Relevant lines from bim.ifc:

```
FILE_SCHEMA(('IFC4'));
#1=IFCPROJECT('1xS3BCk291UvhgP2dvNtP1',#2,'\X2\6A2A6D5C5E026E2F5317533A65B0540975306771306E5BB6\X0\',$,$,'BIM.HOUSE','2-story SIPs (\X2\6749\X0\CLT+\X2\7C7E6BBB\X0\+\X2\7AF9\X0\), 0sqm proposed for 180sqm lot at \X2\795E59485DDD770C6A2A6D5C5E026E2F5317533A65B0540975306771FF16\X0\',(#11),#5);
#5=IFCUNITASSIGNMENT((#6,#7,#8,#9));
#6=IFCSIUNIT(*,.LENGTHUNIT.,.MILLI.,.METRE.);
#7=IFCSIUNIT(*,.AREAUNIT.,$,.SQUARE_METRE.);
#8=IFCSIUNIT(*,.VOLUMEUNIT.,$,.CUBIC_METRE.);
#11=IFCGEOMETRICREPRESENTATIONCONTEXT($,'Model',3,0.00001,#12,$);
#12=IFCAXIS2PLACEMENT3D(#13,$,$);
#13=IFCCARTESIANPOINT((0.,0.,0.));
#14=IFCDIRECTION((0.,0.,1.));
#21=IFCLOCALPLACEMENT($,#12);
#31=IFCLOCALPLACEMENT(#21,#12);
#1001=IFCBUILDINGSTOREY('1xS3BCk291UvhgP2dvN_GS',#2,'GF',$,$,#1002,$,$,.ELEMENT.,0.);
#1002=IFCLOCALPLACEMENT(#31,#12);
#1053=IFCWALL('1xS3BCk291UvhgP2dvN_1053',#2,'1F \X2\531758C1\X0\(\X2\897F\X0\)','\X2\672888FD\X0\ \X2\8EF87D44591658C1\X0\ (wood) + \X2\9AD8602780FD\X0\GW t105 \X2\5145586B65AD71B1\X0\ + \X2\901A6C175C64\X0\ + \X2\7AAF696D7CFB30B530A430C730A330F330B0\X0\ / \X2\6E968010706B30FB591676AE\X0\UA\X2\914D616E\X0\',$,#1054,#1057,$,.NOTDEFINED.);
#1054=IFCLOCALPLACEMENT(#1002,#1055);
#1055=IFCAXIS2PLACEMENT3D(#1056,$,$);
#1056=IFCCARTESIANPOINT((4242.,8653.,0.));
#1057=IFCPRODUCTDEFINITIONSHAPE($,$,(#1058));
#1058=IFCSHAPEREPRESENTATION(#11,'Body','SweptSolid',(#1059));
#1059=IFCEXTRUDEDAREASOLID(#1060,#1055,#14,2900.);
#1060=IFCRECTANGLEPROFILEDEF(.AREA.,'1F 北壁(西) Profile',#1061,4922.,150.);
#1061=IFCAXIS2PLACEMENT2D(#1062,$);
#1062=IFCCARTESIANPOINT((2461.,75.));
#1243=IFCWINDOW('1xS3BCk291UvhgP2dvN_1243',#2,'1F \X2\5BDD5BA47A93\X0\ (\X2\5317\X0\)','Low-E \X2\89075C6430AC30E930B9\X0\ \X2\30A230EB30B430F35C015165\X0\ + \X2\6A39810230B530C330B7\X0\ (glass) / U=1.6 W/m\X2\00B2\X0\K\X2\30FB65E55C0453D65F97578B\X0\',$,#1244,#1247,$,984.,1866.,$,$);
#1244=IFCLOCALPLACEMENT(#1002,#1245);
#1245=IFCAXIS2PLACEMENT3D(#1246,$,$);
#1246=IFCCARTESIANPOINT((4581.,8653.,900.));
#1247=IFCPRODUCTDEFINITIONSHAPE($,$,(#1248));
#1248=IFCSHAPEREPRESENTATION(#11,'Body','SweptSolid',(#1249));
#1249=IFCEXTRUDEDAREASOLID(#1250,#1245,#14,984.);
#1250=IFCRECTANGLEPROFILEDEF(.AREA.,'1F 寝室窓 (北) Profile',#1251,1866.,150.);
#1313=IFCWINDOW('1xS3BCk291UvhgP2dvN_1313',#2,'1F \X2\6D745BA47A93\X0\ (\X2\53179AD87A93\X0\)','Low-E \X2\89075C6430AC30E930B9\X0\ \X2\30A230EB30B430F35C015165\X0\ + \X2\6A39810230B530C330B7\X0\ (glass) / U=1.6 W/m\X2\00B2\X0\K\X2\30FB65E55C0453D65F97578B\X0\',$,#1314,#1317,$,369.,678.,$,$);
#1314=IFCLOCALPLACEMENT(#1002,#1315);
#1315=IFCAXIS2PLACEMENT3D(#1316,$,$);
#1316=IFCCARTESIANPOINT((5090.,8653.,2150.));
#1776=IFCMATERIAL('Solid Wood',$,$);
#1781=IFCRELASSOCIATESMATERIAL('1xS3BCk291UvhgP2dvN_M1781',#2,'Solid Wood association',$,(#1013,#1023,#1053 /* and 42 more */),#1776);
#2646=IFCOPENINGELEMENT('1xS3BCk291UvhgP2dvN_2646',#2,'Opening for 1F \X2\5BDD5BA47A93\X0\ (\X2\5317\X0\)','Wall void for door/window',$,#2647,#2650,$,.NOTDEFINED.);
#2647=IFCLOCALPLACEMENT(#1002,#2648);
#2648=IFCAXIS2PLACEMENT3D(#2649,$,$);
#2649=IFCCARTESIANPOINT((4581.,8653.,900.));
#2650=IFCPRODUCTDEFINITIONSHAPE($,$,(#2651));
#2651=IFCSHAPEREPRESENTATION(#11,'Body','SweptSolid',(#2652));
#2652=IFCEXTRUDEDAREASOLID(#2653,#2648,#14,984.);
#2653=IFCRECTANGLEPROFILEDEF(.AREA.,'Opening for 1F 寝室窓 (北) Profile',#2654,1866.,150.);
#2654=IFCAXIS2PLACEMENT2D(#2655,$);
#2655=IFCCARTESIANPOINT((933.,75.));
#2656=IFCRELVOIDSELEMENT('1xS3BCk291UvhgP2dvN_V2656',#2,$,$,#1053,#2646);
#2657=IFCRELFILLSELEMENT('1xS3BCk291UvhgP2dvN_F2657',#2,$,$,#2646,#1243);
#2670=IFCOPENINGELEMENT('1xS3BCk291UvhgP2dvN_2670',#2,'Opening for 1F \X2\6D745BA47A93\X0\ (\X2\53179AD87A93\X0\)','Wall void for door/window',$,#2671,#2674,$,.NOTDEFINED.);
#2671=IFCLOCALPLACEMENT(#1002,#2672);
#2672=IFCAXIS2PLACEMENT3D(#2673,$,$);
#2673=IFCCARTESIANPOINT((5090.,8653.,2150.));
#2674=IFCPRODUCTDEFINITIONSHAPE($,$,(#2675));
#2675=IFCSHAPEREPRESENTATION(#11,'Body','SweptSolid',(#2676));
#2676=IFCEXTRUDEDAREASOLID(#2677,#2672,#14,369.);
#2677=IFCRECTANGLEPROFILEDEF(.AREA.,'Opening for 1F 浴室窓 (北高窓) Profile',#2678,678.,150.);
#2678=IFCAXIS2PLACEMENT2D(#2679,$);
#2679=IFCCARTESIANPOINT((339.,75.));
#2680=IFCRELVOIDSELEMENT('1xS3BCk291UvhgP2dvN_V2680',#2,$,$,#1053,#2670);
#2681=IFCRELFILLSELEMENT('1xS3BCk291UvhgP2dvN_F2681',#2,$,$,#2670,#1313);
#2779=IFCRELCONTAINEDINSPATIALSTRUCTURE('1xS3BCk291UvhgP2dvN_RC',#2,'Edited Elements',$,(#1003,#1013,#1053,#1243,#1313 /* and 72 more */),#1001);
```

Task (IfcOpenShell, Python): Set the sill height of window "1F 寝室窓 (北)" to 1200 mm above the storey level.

```python
import numpy as np
import ifcopenshell
import ifcopenshell.api.geometry
import ifcopenshell.geom
import ifcopenshell.util.element
import ifcopenshell.util.placement
import ifcopenshell.util.shape
import ifcopenshell.util.unit

model = ifcopenshell.open("bim.ifc")
unit_scale = ifcopenshell.util.unit.calculate_unit_scale(model)

window = model.by_id(1243)
opening = window.FillsVoids[0].RelatingOpeningElement
storey = ifcopenshell.util.element.get_container(window, ifc_class="IfcBuildingStorey")
level = ifcopenshell.util.placement.get_local_placement(storey.ObjectPlacement)[2, 3]

# The opening's origin need not be at the sill, so measure its lowest point.
shape = ifcopenshell.geom.create_shape(ifcopenshell.geom.settings(), opening)
bottom = ifcopenshell.util.shape.get_shape_bottom_elevation(shape, shape.geometry) / unit_scale
dz = level + 1.2 / unit_scale - bottom

shift = np.array([0.0, 0.0, dz])
# The window is not placed relative to its opening, so move both.
for product in (opening, window):
    matrix = ifcopenshell.util.placement.get_local_placement(product.ObjectPlacement)
    matrix[:3, 3] += shift
    ifcopenshell.api.geometry.edit_object_placement(model, product=product, matrix=matrix, is_si=False)

print(f"moved by {dz * unit_scale:+.3f} m")

model.write("bim_edited.ifc")
```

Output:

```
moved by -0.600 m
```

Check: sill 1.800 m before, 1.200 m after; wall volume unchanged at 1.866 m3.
